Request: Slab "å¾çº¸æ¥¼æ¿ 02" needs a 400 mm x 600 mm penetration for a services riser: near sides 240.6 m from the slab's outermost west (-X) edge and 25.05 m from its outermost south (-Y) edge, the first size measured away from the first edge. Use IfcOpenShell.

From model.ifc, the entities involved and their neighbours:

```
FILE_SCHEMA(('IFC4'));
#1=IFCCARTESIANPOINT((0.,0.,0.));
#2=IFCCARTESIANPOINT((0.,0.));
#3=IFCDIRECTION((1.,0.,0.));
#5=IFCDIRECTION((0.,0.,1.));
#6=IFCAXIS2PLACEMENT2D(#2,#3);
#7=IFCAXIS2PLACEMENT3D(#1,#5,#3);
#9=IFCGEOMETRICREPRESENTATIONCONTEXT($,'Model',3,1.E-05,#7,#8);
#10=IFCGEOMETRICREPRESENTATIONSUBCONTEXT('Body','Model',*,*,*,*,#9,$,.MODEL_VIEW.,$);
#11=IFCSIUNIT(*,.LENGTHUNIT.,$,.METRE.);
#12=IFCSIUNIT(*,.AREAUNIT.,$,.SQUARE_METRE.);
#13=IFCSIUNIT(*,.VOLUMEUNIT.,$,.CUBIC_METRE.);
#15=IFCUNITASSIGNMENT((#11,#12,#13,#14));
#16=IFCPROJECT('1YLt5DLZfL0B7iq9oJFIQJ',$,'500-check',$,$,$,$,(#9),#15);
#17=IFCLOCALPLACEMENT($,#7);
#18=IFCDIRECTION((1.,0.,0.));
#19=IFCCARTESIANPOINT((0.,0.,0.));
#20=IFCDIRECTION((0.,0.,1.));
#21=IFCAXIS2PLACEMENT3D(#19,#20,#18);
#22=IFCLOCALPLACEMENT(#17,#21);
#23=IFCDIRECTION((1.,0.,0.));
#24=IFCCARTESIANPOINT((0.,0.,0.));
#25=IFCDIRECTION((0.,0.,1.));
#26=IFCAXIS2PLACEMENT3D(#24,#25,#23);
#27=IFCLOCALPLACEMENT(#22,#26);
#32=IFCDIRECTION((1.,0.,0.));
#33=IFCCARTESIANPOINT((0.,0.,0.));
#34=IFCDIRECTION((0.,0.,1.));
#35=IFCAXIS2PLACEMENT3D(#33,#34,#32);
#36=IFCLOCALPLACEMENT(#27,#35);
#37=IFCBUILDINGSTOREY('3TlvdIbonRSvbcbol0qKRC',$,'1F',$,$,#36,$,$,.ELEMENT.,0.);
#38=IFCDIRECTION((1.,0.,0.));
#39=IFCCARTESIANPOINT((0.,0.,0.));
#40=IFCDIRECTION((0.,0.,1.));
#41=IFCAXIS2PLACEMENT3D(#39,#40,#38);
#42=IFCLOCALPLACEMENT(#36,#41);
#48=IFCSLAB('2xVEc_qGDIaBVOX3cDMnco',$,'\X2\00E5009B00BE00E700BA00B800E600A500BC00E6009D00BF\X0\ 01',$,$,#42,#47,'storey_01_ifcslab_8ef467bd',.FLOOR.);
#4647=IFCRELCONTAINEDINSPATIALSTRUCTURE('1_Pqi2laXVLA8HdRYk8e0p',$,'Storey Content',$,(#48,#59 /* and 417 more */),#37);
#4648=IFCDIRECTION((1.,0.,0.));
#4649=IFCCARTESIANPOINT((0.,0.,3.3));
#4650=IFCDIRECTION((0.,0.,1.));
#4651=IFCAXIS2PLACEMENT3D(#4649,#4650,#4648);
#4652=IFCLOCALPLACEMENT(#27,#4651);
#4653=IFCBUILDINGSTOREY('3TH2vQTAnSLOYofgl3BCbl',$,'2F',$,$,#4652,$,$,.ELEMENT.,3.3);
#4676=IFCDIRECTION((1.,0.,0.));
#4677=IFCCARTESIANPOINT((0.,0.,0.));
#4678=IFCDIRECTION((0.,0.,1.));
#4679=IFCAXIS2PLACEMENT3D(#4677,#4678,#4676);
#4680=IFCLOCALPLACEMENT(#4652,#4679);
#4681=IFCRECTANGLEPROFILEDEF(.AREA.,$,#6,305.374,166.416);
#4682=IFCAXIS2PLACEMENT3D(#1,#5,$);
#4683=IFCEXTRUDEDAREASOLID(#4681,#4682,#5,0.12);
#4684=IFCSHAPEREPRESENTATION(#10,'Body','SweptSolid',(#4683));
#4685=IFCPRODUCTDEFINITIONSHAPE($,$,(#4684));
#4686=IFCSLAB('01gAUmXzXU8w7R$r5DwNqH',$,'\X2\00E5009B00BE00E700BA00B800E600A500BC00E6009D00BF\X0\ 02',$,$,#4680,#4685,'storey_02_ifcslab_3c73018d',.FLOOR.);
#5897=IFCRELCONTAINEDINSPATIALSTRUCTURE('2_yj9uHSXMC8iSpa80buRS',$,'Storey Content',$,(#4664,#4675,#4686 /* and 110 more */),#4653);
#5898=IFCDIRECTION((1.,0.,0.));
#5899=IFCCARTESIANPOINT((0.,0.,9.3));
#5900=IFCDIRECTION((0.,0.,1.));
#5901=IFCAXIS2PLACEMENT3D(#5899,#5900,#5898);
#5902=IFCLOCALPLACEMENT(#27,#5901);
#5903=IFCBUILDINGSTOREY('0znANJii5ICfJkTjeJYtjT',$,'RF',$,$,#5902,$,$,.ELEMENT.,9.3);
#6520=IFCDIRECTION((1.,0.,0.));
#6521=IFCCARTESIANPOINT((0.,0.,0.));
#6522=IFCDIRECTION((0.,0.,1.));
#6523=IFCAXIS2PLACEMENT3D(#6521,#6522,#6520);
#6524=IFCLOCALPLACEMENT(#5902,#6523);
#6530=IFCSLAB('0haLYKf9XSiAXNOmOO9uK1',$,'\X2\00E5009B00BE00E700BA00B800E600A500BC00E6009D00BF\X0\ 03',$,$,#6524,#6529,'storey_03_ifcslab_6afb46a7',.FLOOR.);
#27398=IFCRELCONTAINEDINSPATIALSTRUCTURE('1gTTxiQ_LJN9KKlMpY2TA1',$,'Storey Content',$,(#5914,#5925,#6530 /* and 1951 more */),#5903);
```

```python
import numpy as np
import ifcopenshell
import ifcopenshell.api.feature
import ifcopenshell.api.geometry
import ifcopenshell.api.root
import ifcopenshell.geom
import ifcopenshell.util.placement
import ifcopenshell.util.representation
import ifcopenshell.util.shape
import ifcopenshell.util.unit

model = ifcopenshell.open("model.ifc")
unit_scale = ifcopenshell.util.unit.calculate_unit_scale(model)
settings = ifcopenshell.geom.settings()


def volume(element):
    """Net volume in cubic metres, openings subtracted."""
    shape = ifcopenshell.geom.create_shape(settings, element)
    return ifcopenshell.util.shape.get_volume(shape.geometry)


slab = model.by_guid("01gAUmXzXU8w7R$r5DwNqH")
before = volume(slab)

# Extent in the slab's own axes, in metres. The edges named are its -X and -Y sides.
slab_shape = ifcopenshell.geom.create_shape(settings, slab)
vertices = ifcopenshell.util.shape.get_vertices(slab_shape.geometry)
x_min, y_min, bottom = vertices.min(axis=0)
top = vertices[:, 2].max()

opening = ifcopenshell.api.root.create_entity(model, ifc_class="IfcOpeningElement", name="Services riser opening", predefined_type="OPENING")
context = ifcopenshell.util.representation.get_context(model, "Model", "Body", "MODEL_VIEW")
width, depth = 0.4, 0.6
outline = [(0.0, 0.0), (width, 0.0), (width, depth), (0.0, depth), (0.0, 0.0)]
# Overshoot both faces by 50 mm so the cut is clean.
shape = ifcopenshell.api.geometry.add_slab_representation(
    model, context=context, depth=top - bottom + 0.1, polyline=outline
)
ifcopenshell.api.geometry.assign_representation(model, product=opening, representation=shape)

matrix = ifcopenshell.util.placement.get_local_placement(slab.ObjectPlacement)
matrix[:, 3] = matrix @ np.append(np.array([x_min + 240.6, y_min + 25.05, bottom - 0.05]) / unit_scale, 1.0)
ifcopenshell.api.geometry.edit_object_placement(model, product=opening, matrix=matrix, is_si=False)
ifcopenshell.api.feature.add_feature(model, feature=opening, element=slab)

after = volume(slab)

print(f"slab volume {before:.3f} -> {after:.3f} m3")

model.write("model-out.ifc")
```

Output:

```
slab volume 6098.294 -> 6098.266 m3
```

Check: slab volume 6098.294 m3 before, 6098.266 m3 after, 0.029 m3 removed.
